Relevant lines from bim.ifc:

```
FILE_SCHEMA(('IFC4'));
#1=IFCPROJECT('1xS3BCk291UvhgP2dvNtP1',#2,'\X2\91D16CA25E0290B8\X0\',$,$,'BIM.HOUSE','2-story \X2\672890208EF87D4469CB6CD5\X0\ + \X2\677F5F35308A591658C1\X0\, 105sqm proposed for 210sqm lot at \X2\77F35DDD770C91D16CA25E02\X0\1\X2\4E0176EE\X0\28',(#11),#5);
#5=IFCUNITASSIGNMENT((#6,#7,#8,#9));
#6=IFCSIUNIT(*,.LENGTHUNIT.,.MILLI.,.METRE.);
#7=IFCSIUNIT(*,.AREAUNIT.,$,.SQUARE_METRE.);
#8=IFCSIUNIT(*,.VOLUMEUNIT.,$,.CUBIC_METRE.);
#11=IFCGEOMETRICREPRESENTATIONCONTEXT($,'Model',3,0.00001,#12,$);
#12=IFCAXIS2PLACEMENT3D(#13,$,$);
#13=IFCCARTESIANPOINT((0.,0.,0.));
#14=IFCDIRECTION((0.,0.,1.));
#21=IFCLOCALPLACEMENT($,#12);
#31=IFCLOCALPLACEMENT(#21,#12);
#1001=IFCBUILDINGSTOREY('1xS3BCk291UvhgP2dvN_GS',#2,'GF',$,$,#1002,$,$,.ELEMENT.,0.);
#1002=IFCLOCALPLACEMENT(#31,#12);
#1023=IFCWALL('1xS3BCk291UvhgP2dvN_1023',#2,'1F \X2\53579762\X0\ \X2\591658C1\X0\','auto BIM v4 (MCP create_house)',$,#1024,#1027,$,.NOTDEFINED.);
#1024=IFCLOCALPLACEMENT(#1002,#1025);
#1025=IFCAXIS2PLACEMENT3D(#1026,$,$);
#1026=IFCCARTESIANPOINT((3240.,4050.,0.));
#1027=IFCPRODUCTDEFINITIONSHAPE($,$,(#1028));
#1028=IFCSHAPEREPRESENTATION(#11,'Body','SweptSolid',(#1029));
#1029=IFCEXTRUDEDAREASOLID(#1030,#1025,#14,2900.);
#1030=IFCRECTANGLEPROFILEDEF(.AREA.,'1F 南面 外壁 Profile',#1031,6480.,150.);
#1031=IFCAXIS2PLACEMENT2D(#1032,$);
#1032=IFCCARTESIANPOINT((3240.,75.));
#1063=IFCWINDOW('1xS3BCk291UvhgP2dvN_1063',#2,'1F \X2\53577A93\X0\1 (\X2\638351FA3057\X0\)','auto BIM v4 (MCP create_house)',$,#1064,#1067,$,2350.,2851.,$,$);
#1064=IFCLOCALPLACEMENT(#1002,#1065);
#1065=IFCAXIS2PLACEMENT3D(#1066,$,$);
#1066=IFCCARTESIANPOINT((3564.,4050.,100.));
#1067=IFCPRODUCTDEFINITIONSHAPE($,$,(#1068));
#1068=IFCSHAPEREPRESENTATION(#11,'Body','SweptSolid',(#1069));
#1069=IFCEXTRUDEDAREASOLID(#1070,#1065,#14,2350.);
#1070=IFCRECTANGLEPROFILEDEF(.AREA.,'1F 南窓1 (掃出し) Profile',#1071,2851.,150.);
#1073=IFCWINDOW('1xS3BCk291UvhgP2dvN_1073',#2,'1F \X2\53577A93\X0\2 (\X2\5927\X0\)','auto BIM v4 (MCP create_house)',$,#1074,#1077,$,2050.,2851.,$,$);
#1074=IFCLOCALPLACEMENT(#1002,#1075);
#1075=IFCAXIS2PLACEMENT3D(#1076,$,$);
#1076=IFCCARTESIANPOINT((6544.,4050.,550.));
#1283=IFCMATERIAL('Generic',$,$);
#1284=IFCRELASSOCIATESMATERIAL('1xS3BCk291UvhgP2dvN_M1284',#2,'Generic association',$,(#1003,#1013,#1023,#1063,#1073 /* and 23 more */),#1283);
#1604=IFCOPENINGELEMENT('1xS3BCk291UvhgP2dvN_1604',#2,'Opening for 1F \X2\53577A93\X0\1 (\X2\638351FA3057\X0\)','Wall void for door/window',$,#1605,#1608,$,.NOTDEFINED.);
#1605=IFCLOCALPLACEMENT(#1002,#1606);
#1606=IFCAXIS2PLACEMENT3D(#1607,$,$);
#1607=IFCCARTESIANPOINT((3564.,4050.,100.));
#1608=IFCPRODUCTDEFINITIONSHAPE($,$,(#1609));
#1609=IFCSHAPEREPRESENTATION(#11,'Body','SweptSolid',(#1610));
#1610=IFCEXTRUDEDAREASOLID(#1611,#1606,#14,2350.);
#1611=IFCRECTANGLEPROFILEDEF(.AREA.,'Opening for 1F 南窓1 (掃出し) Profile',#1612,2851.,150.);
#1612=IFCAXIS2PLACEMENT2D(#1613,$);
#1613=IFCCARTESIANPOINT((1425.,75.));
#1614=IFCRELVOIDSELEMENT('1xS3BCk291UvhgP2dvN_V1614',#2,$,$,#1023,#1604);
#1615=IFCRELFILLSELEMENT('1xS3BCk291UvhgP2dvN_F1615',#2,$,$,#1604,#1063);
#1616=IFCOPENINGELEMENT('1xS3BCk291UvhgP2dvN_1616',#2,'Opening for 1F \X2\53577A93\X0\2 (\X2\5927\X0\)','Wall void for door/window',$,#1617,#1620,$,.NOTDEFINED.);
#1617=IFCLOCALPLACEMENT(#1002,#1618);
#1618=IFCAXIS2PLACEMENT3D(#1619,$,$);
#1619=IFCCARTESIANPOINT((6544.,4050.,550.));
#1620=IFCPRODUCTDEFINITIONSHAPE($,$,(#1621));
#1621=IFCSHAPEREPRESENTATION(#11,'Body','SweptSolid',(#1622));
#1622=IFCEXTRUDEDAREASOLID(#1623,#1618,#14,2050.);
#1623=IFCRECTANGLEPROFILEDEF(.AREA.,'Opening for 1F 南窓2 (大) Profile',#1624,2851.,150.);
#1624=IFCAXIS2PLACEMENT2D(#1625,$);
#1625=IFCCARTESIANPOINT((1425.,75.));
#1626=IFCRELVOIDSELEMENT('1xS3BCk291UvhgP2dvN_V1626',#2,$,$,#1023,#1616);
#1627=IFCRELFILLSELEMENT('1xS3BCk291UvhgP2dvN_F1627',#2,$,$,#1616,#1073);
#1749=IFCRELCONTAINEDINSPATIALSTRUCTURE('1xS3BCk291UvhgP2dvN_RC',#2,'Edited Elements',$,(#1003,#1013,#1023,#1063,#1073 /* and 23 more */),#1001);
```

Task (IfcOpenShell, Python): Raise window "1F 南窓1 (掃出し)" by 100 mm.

```python
import numpy as np
import ifcopenshell
import ifcopenshell.api.geometry
import ifcopenshell.util.placement
import ifcopenshell.util.unit

model = ifcopenshell.open("bim.ifc")
unit_scale = ifcopenshell.util.unit.calculate_unit_scale(model)

window = model.by_guid("1xS3BCk291UvhgP2dvN_1063")
opening = window.FillsVoids[0].RelatingOpeningElement
dz = 0.1 / unit_scale

shift = np.array([0.0, 0.0, dz])
# The window is not placed relative to its opening, so move both.
for product in (opening, window):
    matrix = ifcopenshell.util.placement.get_local_placement(product.ObjectPlacement)
    matrix[:3, 3] += shift
    ifcopenshell.api.geometry.edit_object_placement(model, product=product, matrix=matrix, is_si=False)

print(f"moved by {dz * unit_scale:+.3f} m")

model.write("bim_rev.ifc")
```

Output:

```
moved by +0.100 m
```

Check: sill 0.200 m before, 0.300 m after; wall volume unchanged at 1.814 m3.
